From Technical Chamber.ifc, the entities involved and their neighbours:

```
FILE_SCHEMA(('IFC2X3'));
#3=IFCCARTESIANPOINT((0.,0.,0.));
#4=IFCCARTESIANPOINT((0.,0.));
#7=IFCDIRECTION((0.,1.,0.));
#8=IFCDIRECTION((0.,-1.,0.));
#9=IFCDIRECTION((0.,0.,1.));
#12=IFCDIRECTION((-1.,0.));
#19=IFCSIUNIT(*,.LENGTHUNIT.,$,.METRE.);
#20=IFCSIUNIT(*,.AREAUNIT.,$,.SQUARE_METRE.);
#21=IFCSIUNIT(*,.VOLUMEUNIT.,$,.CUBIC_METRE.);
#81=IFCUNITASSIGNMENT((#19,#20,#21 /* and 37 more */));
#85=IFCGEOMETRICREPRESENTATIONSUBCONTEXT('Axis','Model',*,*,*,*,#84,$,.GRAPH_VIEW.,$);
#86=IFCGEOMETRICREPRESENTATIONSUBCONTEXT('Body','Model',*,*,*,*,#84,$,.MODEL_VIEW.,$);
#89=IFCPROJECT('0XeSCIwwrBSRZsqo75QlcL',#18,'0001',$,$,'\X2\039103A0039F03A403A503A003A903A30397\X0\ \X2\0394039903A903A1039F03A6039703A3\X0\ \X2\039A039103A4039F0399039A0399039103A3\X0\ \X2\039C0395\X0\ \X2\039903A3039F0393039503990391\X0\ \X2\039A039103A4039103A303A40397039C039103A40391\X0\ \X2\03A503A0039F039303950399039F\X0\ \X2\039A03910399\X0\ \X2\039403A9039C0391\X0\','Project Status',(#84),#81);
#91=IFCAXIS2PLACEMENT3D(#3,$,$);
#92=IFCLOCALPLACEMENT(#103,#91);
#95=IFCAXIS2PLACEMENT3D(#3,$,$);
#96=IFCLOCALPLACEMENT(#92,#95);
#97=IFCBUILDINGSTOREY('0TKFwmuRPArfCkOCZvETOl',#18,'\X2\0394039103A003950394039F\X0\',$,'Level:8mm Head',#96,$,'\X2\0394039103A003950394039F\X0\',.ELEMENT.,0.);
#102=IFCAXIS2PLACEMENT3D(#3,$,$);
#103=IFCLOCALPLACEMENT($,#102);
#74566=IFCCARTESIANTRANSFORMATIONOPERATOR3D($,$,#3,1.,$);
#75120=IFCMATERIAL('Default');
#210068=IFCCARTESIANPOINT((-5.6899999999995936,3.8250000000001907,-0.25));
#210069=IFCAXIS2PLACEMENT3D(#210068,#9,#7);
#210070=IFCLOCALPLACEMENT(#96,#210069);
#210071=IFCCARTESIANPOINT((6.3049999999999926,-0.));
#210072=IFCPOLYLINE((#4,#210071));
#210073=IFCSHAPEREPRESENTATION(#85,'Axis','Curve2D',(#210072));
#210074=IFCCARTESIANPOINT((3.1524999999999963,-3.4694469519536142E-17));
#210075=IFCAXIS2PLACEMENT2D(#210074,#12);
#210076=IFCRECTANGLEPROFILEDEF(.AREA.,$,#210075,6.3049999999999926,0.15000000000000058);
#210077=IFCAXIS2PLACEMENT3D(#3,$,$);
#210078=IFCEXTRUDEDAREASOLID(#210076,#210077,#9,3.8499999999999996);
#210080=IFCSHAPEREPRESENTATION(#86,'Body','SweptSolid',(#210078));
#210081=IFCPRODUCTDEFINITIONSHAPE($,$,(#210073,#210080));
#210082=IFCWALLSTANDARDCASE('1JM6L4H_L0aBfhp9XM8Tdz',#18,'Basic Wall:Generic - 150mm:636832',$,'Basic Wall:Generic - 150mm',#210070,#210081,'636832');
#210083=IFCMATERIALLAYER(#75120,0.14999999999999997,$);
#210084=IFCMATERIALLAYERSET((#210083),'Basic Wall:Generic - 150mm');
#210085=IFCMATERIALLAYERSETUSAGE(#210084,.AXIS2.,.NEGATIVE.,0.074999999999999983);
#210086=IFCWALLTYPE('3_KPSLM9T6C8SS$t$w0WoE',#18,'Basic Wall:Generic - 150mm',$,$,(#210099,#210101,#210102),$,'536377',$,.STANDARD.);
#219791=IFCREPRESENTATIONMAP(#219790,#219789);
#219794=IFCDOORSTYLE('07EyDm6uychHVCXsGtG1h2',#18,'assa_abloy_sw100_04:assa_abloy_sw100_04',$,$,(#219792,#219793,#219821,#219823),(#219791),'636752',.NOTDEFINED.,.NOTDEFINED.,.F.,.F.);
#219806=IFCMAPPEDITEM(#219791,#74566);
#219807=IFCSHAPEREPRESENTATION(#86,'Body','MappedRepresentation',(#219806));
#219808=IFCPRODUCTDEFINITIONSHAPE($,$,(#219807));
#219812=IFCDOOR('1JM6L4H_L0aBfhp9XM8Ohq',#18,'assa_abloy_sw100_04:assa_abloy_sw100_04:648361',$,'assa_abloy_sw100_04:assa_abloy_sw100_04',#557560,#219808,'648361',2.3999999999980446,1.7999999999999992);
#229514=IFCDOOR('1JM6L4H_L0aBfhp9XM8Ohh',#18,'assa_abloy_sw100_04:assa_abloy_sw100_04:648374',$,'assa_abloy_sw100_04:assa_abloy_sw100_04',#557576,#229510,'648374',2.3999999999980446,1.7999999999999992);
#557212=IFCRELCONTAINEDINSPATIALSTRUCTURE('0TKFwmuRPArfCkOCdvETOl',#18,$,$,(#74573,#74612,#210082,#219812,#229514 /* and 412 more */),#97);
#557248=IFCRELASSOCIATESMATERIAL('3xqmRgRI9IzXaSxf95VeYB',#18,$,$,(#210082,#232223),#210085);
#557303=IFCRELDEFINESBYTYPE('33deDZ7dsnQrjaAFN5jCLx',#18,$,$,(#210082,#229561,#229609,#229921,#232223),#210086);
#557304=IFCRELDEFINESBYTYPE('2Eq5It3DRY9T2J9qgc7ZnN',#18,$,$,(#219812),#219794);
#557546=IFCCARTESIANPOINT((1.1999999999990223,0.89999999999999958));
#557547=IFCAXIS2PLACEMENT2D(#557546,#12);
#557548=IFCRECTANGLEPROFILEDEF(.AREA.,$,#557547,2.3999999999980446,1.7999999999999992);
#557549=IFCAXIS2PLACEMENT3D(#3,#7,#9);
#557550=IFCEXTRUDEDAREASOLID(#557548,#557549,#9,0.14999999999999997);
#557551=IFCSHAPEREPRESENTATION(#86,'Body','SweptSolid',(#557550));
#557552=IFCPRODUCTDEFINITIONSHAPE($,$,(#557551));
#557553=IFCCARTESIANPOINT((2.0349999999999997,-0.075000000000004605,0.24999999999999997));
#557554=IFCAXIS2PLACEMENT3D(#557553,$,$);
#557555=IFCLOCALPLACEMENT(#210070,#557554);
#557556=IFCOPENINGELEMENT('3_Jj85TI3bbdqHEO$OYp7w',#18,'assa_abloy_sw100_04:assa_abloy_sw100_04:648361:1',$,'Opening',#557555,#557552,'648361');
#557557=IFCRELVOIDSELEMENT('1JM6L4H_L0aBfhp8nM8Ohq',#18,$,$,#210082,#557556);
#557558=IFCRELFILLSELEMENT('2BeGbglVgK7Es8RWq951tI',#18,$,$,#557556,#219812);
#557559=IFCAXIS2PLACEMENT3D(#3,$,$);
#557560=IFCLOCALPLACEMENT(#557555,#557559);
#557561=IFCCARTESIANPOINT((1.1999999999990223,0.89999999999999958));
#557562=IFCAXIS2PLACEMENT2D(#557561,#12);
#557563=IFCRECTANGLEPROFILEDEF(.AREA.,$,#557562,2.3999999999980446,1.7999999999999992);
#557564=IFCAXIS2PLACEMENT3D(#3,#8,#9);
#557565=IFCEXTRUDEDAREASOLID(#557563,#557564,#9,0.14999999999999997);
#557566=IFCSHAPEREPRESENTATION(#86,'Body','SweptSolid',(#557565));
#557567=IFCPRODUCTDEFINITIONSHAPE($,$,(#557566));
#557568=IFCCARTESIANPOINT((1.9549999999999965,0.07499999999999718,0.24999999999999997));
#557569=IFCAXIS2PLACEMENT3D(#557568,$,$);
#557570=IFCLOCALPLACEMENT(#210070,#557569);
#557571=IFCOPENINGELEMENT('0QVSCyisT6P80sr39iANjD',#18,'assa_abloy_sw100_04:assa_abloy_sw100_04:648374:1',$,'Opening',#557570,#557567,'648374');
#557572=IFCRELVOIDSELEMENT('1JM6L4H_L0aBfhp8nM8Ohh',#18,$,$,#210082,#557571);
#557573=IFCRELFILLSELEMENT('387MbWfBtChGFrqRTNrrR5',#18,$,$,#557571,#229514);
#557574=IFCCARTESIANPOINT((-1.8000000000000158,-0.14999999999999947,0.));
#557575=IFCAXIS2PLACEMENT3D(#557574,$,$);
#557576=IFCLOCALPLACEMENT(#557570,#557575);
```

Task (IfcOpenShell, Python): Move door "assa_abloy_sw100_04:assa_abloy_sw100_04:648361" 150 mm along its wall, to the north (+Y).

```python
import ifcopenshell
import ifcopenshell.api.geometry
import ifcopenshell.util.placement
import ifcopenshell.util.unit

model = ifcopenshell.open("Technical Chamber.ifc")
unit_scale = ifcopenshell.util.unit.calculate_unit_scale(model)

door = model.by_id(219812)
opening = door.FillsVoids[0].RelatingOpeningElement
wall = opening.VoidsElements[0].RelatingBuildingElement

wall_matrix = ifcopenshell.util.placement.get_local_placement(wall.ObjectPlacement)
shift = wall_matrix[:3, 0] * 0.15 / unit_scale
before = ifcopenshell.util.placement.get_local_placement(door.ObjectPlacement)[:3, 3].copy()

# The door is placed relative to its opening, so it follows when the opening moves.
matrix = ifcopenshell.util.placement.get_local_placement(opening.ObjectPlacement)
matrix[:3, 3] += shift
ifcopenshell.api.geometry.edit_object_placement(
    model, product=opening, matrix=matrix, is_si=False, should_transform_children=True
)

after = ifcopenshell.util.placement.get_local_placement(door.ObjectPlacement)[:3, 3]
print("door moved by", (after - before).round(3) + 0.0)

model.write("Technical Chamber_edited.ifc")
```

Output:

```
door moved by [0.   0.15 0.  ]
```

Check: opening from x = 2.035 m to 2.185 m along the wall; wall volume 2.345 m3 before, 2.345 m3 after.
